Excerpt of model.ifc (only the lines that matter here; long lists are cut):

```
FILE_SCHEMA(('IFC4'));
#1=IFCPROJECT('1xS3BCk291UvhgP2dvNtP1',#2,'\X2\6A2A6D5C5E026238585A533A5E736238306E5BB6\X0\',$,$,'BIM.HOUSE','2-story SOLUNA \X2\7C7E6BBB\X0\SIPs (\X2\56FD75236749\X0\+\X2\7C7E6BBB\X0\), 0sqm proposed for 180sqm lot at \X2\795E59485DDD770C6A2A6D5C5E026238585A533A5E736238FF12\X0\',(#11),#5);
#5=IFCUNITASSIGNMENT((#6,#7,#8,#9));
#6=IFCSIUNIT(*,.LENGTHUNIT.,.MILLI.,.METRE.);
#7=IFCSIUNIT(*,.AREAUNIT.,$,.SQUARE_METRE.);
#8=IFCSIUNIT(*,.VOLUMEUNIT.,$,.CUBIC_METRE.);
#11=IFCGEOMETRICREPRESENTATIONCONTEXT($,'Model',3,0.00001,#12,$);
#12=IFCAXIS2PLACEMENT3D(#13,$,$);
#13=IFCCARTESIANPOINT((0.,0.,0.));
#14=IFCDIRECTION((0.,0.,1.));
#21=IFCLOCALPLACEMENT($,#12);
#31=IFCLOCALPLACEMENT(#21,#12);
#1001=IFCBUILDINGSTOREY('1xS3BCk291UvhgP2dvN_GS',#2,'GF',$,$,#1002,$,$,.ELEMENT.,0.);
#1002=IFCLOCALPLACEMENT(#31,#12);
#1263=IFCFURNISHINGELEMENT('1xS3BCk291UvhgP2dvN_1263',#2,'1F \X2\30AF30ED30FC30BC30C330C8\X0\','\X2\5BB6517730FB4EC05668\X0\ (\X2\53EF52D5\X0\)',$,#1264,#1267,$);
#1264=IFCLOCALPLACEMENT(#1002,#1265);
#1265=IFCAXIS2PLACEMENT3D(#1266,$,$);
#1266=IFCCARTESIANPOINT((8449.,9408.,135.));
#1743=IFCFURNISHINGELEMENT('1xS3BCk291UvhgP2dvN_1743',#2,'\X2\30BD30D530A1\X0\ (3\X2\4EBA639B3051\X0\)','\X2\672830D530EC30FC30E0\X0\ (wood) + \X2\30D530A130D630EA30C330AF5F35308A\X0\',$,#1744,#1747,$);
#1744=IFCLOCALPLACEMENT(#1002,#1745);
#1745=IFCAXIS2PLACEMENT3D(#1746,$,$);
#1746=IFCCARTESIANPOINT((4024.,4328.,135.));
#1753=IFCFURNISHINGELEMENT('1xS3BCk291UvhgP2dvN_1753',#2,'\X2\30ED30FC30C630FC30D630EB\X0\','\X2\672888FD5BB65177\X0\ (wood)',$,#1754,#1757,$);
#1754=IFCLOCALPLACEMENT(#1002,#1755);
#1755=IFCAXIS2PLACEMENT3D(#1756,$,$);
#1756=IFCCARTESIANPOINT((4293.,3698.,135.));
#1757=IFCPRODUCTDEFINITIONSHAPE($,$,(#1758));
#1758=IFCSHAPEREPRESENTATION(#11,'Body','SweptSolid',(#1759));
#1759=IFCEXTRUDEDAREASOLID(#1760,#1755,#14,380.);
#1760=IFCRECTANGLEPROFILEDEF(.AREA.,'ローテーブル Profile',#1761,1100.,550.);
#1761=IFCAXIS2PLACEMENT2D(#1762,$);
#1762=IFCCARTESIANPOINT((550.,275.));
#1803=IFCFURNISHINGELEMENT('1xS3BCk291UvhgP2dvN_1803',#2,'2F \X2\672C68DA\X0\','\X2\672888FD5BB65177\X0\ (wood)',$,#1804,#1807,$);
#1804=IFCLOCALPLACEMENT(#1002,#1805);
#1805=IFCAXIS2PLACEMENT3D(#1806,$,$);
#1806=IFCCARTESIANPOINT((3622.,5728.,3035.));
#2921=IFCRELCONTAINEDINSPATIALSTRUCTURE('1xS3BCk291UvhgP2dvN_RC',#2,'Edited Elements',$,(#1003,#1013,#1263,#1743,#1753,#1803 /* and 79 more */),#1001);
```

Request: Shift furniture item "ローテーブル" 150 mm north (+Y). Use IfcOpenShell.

```python
import ifcopenshell
import ifcopenshell.api.geometry
import ifcopenshell.util.placement

model = ifcopenshell.open("model.ifc")

item = model.by_guid("1xS3BCk291UvhgP2dvN_1753")
matrix = ifcopenshell.util.placement.get_local_placement(item.ObjectPlacement)
matrix[1, 3] += 150.0
ifcopenshell.api.geometry.edit_object_placement(model, product=item, matrix=matrix, is_si=False)

print(ifcopenshell.util.placement.get_local_placement(item.ObjectPlacement).round(3) + 0.0)

model.write("model_rev.ifc")
```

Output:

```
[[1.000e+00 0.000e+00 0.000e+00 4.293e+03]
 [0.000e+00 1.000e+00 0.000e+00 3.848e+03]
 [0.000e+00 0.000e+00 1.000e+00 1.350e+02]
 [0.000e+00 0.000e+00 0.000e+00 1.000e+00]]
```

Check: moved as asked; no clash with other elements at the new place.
